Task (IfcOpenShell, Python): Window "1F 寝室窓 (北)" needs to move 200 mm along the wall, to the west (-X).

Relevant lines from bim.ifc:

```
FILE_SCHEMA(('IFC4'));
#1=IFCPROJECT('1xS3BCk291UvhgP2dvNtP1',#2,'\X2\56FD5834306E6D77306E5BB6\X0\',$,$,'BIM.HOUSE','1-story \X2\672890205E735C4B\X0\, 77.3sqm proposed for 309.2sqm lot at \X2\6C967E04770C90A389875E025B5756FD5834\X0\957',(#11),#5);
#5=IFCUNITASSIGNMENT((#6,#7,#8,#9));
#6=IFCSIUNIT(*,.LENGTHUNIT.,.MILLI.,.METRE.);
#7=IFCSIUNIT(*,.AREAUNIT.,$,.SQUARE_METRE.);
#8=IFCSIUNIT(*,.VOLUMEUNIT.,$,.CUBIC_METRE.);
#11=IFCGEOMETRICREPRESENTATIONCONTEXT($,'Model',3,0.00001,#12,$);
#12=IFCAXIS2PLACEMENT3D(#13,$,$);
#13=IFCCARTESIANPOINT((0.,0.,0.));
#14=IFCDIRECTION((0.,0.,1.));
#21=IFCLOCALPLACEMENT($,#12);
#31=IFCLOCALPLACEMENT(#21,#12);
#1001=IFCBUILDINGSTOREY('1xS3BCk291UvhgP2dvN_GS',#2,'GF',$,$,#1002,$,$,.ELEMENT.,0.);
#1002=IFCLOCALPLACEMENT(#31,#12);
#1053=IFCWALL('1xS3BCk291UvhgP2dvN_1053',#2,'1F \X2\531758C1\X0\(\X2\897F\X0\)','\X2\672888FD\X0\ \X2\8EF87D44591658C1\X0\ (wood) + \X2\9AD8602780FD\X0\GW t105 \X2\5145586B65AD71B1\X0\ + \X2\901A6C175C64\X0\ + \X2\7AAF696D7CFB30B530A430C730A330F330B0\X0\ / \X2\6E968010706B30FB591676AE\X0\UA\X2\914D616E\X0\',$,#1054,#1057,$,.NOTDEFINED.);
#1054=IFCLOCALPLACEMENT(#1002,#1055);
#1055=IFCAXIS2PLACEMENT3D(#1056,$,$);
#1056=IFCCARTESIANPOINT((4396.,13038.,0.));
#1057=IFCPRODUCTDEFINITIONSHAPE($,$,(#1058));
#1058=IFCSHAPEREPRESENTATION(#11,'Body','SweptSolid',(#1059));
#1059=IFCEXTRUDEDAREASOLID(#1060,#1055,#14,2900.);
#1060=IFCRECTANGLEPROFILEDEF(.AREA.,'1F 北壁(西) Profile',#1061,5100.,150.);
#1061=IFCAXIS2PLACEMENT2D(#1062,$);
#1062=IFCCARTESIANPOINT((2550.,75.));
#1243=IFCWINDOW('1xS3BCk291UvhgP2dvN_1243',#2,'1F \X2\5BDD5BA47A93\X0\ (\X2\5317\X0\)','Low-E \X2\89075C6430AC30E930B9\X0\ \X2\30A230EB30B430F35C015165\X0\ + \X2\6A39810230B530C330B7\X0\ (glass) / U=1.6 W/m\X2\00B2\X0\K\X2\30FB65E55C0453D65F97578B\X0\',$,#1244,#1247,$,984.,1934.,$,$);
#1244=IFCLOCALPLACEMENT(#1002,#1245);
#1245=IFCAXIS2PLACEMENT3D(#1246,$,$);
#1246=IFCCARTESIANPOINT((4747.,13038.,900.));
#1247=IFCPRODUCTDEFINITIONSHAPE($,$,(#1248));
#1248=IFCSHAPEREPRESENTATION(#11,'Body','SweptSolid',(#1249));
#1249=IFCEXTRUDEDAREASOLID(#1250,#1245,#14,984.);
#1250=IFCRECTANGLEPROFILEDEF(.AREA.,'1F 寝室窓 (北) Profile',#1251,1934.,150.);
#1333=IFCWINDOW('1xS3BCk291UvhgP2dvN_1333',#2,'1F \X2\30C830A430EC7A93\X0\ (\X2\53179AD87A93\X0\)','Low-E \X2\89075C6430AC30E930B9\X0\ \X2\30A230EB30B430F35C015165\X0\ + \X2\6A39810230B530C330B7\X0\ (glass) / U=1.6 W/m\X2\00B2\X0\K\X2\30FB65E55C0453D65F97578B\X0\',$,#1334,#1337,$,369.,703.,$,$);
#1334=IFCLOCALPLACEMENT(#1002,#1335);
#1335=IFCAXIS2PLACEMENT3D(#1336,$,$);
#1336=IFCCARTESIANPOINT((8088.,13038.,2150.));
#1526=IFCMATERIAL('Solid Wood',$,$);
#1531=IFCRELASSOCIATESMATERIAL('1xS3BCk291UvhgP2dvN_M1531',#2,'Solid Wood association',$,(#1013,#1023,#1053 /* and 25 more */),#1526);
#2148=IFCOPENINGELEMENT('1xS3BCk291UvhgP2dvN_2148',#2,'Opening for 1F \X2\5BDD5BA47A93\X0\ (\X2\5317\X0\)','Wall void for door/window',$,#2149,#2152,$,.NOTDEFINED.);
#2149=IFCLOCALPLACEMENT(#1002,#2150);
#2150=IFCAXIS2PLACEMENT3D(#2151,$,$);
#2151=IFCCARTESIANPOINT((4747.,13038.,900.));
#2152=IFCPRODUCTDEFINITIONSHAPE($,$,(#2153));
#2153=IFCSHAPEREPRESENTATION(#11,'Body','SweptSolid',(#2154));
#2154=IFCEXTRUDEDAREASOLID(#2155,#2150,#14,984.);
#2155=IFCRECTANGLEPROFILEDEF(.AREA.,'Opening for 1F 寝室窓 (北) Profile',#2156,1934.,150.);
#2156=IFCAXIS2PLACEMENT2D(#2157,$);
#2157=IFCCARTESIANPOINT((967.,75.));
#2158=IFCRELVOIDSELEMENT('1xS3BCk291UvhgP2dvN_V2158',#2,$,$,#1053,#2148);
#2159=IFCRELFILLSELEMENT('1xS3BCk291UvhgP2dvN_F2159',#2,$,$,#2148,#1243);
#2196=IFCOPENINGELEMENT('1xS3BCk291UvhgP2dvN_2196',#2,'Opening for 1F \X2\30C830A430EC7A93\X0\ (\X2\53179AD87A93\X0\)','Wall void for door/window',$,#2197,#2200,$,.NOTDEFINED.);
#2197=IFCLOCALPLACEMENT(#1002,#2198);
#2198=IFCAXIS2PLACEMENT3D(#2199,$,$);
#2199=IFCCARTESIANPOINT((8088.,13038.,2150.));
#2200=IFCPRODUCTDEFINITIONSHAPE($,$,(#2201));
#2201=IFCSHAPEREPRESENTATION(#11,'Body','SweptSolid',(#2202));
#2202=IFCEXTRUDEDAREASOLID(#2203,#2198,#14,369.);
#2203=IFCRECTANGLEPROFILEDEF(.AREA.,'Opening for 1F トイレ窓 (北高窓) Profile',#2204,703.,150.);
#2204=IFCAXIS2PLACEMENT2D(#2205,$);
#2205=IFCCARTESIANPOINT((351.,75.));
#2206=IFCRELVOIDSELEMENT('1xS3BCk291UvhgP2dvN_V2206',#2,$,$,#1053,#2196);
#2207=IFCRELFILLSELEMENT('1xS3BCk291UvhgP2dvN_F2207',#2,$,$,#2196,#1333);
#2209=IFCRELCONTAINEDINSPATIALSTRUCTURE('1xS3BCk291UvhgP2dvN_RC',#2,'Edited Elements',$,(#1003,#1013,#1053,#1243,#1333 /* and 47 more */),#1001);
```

```python
import ifcopenshell
import ifcopenshell.api.geometry
import ifcopenshell.util.placement
import ifcopenshell.util.unit

model = ifcopenshell.open("bim.ifc")
unit_scale = ifcopenshell.util.unit.calculate_unit_scale(model)

window = model.by_guid("1xS3BCk291UvhgP2dvN_1243")
opening = window.FillsVoids[0].RelatingOpeningElement
wall = opening.VoidsElements[0].RelatingBuildingElement

wall_matrix = ifcopenshell.util.placement.get_local_placement(wall.ObjectPlacement)
shift = wall_matrix[:3, 0] * -0.2 / unit_scale
before = ifcopenshell.util.placement.get_local_placement(window.ObjectPlacement)[:3, 3].copy()

# The window is not placed relative to its opening, so move both.
for product in (opening, window):
    matrix = ifcopenshell.util.placement.get_local_placement(product.ObjectPlacement)
    matrix[:3, 3] += shift
    ifcopenshell.api.geometry.edit_object_placement(model, product=product, matrix=matrix, is_si=False)

after = ifcopenshell.util.placement.get_local_placement(window.ObjectPlacement)[:3, 3]
print("window moved by", (after - before).round(3) + 0.0)

model.write("bim_v2.ifc")
```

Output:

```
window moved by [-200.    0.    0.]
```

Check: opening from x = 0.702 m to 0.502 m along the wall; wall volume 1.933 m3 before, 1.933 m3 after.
